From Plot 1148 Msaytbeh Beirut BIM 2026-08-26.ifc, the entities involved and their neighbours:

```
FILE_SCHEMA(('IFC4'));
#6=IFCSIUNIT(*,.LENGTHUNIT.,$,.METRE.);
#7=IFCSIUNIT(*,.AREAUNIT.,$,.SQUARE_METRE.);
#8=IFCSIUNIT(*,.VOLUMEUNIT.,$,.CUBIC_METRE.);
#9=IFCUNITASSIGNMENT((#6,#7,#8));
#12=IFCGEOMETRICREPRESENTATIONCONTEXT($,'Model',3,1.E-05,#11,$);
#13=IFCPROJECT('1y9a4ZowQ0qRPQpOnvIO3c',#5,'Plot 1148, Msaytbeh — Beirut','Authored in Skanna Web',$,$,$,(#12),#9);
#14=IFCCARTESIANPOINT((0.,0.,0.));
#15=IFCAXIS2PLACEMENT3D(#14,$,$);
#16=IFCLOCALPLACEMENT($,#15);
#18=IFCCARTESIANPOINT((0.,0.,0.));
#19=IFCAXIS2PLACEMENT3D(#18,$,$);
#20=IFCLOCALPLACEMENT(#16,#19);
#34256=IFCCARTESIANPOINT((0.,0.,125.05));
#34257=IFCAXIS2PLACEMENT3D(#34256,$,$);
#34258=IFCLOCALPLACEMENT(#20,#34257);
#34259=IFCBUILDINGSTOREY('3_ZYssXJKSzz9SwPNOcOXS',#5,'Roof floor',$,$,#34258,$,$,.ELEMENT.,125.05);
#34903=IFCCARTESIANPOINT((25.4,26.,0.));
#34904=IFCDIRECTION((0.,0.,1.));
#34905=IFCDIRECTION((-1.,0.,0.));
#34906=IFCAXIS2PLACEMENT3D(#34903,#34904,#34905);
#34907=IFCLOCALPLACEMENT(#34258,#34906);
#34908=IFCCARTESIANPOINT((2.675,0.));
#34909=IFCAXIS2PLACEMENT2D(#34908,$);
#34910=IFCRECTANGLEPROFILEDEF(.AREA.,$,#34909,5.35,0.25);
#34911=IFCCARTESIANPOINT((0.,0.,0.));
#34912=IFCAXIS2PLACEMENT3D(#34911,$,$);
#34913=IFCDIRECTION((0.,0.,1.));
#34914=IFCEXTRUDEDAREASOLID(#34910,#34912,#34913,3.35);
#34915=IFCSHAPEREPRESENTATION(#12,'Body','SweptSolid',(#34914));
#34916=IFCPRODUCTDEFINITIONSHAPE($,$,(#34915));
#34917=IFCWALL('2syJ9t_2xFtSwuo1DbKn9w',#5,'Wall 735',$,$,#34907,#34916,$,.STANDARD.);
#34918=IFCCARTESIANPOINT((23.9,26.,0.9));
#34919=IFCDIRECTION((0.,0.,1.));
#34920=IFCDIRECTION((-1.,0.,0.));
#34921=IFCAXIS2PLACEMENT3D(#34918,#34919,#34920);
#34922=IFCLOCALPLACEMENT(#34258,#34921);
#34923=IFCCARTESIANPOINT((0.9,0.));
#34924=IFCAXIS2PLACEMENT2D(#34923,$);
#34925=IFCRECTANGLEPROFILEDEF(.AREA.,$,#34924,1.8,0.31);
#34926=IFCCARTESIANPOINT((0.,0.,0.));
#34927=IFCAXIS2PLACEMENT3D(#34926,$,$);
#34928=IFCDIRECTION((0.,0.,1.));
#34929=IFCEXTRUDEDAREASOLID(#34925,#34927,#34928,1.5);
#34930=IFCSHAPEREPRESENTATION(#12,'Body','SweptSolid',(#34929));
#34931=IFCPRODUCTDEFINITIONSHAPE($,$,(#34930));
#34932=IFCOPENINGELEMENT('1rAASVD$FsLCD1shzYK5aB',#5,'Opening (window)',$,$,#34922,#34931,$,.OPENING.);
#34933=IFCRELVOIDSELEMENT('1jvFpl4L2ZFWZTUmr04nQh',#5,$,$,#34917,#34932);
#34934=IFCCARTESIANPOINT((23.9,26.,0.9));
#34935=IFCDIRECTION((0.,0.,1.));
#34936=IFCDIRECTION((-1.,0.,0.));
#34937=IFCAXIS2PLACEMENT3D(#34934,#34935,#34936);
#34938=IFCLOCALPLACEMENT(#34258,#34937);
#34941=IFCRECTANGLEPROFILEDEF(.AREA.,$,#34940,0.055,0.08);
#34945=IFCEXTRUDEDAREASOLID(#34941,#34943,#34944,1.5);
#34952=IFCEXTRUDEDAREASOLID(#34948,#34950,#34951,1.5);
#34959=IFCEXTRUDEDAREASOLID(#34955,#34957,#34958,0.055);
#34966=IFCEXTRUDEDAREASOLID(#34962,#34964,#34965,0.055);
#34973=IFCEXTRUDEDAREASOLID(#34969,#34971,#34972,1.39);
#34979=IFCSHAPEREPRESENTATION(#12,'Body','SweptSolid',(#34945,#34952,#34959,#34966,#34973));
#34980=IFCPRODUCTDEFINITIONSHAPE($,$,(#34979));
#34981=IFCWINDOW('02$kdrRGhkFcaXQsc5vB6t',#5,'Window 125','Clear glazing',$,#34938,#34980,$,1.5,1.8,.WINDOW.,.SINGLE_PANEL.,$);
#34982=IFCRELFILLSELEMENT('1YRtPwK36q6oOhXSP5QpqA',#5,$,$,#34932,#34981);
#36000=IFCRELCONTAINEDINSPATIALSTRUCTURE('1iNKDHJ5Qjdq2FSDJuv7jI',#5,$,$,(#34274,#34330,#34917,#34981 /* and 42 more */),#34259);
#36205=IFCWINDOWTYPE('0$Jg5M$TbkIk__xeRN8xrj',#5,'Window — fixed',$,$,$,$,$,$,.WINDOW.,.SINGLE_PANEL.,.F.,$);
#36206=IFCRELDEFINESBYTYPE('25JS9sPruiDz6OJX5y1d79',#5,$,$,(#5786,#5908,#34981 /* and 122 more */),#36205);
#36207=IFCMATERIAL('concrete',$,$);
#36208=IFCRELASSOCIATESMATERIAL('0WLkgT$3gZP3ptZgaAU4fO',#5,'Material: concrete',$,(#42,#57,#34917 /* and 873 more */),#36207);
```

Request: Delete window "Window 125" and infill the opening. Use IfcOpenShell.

```python
import ifcopenshell
import ifcopenshell.api.feature
import ifcopenshell.api.root
import ifcopenshell.geom
import ifcopenshell.util.shape

model = ifcopenshell.open("Plot 1148 Msaytbeh Beirut BIM 2026-08-26.ifc")
settings = ifcopenshell.geom.settings()


def volume(element):
    """Net volume in cubic metres, openings subtracted."""
    shape = ifcopenshell.geom.create_shape(settings, element)
    return ifcopenshell.util.shape.get_volume(shape.geometry)


window = model.by_guid("02$kdrRGhkFcaXQsc5vB6t")
opening = window.FillsVoids[0].RelatingOpeningElement
wall = opening.VoidsElements[0].RelatingBuildingElement
before = volume(wall)

ifcopenshell.api.root.remove_product(model, product=window)
ifcopenshell.api.feature.remove_feature(model, feature=opening)

after = volume(wall)

print(f"wall volume {before:.3f} -> {after:.3f} m3")

model.write("Plot 1148 Msaytbeh Beirut BIM 2026-08-26_rev.ifc")
```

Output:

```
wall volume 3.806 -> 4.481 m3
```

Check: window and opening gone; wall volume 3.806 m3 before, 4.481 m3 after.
